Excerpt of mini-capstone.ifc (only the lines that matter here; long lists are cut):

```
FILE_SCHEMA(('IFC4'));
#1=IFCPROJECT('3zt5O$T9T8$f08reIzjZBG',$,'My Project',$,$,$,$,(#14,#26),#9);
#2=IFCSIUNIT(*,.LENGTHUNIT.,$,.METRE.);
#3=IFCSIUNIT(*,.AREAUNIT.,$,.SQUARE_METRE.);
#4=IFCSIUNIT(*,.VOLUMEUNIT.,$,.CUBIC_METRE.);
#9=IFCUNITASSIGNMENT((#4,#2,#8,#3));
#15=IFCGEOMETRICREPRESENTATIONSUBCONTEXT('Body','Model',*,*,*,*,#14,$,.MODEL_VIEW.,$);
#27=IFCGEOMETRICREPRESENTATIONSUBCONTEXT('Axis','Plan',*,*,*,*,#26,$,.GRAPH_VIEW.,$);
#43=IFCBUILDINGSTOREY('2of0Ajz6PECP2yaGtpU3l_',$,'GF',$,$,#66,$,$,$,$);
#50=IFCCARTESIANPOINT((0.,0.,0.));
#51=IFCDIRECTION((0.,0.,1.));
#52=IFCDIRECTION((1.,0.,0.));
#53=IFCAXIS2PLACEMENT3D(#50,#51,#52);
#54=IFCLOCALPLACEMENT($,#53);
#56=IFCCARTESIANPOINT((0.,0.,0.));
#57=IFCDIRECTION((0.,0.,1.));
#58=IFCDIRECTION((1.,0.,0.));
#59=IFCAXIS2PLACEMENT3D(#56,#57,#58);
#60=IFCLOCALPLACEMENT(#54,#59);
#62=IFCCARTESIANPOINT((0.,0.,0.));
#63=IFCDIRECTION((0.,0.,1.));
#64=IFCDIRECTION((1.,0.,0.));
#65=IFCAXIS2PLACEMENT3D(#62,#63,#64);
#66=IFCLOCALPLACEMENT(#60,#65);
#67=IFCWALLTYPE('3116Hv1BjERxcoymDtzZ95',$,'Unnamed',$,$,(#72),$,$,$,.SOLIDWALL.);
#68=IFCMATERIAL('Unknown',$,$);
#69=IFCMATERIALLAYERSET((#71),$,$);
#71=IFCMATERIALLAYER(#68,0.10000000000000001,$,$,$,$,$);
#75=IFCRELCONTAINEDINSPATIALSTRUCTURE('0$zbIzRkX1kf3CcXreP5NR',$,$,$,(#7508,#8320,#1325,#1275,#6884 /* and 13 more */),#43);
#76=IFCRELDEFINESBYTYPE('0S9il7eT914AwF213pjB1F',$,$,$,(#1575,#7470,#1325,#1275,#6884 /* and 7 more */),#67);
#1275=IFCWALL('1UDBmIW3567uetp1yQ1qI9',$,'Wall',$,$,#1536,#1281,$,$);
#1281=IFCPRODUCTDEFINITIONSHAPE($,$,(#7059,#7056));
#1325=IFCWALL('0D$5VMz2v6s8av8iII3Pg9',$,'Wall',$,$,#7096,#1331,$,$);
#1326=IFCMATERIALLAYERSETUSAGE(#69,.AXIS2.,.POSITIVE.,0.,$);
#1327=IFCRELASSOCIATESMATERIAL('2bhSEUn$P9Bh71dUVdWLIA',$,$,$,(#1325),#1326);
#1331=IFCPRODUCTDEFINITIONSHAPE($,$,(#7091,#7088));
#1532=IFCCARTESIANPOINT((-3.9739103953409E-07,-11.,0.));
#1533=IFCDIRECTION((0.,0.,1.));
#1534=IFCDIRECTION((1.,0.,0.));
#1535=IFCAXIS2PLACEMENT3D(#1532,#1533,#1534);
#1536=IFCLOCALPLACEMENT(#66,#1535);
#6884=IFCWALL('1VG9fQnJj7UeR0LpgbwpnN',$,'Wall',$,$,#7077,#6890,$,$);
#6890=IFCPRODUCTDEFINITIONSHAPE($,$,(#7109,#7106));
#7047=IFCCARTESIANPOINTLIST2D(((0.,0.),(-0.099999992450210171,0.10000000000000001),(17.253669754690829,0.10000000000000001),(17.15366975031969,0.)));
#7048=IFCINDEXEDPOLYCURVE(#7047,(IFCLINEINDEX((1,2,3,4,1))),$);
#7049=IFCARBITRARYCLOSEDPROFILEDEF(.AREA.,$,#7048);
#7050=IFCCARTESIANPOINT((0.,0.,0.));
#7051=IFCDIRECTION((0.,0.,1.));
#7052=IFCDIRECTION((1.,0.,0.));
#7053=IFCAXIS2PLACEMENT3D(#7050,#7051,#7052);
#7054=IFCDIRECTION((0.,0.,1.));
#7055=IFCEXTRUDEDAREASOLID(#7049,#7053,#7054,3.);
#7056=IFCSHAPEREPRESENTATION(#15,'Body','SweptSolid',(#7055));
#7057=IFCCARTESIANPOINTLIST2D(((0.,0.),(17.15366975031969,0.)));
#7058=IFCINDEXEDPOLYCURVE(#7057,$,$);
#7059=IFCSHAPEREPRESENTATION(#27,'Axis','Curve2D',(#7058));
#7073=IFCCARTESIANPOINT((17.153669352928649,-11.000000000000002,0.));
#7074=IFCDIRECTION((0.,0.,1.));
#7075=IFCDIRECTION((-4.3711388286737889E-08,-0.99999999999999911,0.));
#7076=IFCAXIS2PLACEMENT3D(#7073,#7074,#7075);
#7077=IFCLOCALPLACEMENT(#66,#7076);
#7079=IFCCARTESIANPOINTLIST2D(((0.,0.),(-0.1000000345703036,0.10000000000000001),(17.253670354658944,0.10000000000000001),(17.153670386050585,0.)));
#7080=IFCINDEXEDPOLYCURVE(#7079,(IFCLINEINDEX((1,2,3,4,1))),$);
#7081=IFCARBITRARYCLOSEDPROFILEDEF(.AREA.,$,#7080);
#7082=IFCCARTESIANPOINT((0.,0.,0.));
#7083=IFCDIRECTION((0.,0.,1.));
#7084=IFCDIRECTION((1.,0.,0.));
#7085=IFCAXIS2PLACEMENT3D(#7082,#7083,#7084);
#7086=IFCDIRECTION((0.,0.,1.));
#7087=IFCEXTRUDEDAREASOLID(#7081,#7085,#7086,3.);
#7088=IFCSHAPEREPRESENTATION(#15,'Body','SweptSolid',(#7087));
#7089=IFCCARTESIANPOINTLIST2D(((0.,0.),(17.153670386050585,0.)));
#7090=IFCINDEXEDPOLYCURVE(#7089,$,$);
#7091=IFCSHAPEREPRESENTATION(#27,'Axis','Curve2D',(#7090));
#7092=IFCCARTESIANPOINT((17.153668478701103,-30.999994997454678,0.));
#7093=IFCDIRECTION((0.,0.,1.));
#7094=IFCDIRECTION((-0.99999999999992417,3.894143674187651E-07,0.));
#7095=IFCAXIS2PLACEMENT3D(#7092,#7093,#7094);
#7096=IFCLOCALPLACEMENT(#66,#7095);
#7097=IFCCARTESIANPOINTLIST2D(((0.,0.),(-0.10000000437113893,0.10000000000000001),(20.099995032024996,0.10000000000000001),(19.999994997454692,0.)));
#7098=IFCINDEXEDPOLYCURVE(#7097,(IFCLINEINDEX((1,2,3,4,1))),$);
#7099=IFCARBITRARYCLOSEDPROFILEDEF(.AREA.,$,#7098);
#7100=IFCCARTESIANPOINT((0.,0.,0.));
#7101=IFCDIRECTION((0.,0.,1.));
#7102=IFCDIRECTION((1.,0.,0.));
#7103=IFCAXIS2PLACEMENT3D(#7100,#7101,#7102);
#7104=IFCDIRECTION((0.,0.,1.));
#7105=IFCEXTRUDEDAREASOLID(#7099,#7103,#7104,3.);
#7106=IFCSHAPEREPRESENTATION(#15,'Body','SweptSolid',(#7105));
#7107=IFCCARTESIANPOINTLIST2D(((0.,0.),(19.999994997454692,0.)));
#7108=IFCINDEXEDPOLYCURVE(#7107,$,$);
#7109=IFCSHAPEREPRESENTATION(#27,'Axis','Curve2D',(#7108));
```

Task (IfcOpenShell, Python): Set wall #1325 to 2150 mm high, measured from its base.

```python
import ifcopenshell
import ifcopenshell.geom
import ifcopenshell.util.representation
import ifcopenshell.util.shape
import ifcopenshell.util.unit

model = ifcopenshell.open("mini-capstone.ifc")
unit_scale = ifcopenshell.util.unit.calculate_unit_scale(model)
settings = ifcopenshell.geom.settings()


def volume(element):
    """Net volume in cubic metres, openings subtracted."""
    shape = ifcopenshell.geom.create_shape(settings, element)
    return ifcopenshell.util.shape.get_volume(shape.geometry)


wall = model.by_guid("0D$5VMz2v6s8av8iII3Pg9")
before = volume(wall)

body = ifcopenshell.util.representation.get_representation(wall, "Model", "Body")
solid = body.Items[0]
old_height = solid.Depth
solid.Depth = 2.15 / unit_scale
after = volume(wall)

print(f"height {old_height:g} -> {solid.Depth:g}, volume {before:.3f} -> {after:.3f} m3")

model.write("mini-capstone_edited.ifc")
```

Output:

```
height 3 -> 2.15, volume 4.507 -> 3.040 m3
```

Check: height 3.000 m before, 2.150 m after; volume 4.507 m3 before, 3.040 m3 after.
